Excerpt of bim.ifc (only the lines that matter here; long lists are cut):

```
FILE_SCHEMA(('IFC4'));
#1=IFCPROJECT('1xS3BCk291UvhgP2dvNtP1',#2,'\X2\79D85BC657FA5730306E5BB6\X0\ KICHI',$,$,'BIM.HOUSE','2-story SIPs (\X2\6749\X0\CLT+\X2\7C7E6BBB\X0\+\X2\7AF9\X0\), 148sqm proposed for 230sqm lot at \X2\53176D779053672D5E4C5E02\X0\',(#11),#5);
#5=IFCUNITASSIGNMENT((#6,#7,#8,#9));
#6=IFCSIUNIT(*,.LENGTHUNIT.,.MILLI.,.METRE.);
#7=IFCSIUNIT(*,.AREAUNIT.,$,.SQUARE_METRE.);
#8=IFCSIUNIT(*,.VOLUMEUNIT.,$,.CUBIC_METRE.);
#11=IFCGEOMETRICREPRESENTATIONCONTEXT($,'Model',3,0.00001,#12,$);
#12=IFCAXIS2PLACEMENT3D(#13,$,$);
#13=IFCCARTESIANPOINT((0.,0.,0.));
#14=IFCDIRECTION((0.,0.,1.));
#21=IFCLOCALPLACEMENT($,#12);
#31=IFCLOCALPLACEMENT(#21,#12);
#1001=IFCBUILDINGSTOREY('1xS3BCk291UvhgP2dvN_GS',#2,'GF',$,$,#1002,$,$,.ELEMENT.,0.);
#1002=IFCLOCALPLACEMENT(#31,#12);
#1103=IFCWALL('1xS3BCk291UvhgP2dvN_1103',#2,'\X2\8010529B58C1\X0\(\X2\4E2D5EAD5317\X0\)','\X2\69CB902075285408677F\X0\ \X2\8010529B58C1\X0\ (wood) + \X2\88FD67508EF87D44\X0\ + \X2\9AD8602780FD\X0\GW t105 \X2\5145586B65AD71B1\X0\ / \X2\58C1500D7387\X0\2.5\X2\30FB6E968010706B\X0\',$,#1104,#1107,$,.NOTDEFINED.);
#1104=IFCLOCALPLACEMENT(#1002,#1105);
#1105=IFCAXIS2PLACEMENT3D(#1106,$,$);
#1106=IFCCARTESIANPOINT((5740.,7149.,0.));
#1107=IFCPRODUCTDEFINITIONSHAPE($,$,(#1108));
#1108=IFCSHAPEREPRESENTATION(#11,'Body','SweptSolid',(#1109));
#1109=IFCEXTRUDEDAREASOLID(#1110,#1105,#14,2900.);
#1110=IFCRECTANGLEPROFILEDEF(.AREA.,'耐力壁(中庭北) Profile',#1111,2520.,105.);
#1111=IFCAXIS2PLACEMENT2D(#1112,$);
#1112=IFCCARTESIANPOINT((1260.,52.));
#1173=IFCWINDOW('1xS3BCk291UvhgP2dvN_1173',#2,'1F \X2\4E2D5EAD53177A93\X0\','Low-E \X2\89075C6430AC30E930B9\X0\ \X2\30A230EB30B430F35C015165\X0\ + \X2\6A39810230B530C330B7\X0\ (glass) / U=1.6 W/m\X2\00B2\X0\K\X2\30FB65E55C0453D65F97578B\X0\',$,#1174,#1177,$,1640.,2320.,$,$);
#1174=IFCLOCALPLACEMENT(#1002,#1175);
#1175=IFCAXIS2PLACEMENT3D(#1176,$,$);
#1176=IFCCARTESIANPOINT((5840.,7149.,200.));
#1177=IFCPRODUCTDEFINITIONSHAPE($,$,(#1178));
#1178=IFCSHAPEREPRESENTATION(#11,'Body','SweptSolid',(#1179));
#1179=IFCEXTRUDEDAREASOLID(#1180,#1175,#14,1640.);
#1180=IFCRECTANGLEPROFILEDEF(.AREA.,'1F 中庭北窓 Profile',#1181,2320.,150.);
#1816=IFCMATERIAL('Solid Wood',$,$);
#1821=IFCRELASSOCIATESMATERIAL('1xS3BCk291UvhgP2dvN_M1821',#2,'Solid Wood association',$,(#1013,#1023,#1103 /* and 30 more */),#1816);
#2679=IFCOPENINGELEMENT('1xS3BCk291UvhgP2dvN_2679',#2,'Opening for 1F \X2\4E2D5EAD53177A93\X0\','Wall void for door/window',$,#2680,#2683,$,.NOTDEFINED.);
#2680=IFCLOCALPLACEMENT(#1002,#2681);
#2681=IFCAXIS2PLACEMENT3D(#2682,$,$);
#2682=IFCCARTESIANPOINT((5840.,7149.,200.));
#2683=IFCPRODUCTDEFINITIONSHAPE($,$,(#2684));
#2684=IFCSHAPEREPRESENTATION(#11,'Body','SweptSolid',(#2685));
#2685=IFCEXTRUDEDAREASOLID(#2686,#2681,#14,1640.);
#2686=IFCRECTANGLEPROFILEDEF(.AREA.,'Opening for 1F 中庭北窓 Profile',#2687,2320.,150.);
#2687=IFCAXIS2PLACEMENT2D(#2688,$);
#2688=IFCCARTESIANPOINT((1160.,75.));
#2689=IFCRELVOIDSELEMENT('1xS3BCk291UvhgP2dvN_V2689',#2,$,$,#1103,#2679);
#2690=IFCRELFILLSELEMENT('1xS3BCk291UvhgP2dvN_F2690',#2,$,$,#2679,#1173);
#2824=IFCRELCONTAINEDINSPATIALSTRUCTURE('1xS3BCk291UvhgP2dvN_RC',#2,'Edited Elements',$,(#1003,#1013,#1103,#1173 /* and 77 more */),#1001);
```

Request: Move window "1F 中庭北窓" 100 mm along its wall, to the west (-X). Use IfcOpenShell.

```python
import ifcopenshell
import ifcopenshell.api.geometry
import ifcopenshell.util.placement
import ifcopenshell.util.unit

model = ifcopenshell.open("bim.ifc")
unit_scale = ifcopenshell.util.unit.calculate_unit_scale(model)

window = model.by_guid("1xS3BCk291UvhgP2dvN_1173")
opening = window.FillsVoids[0].RelatingOpeningElement
wall = opening.VoidsElements[0].RelatingBuildingElement

wall_matrix = ifcopenshell.util.placement.get_local_placement(wall.ObjectPlacement)
shift = wall_matrix[:3, 0] * -0.1 / unit_scale
before = ifcopenshell.util.placement.get_local_placement(window.ObjectPlacement)[:3, 3].copy()

# The window is not placed relative to its opening, so move both.
for product in (opening, window):
    matrix = ifcopenshell.util.placement.get_local_placement(product.ObjectPlacement)
    matrix[:3, 3] += shift
    ifcopenshell.api.geometry.edit_object_placement(model, product=product, matrix=matrix, is_si=False)

after = ifcopenshell.util.placement.get_local_placement(window.ObjectPlacement)[:3, 3]
print("window moved by", (after - before).round(3) + 0.0)

model.write("bim-out.ifc")
```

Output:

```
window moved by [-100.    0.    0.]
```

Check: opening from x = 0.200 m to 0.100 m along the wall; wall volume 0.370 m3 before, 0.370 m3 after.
